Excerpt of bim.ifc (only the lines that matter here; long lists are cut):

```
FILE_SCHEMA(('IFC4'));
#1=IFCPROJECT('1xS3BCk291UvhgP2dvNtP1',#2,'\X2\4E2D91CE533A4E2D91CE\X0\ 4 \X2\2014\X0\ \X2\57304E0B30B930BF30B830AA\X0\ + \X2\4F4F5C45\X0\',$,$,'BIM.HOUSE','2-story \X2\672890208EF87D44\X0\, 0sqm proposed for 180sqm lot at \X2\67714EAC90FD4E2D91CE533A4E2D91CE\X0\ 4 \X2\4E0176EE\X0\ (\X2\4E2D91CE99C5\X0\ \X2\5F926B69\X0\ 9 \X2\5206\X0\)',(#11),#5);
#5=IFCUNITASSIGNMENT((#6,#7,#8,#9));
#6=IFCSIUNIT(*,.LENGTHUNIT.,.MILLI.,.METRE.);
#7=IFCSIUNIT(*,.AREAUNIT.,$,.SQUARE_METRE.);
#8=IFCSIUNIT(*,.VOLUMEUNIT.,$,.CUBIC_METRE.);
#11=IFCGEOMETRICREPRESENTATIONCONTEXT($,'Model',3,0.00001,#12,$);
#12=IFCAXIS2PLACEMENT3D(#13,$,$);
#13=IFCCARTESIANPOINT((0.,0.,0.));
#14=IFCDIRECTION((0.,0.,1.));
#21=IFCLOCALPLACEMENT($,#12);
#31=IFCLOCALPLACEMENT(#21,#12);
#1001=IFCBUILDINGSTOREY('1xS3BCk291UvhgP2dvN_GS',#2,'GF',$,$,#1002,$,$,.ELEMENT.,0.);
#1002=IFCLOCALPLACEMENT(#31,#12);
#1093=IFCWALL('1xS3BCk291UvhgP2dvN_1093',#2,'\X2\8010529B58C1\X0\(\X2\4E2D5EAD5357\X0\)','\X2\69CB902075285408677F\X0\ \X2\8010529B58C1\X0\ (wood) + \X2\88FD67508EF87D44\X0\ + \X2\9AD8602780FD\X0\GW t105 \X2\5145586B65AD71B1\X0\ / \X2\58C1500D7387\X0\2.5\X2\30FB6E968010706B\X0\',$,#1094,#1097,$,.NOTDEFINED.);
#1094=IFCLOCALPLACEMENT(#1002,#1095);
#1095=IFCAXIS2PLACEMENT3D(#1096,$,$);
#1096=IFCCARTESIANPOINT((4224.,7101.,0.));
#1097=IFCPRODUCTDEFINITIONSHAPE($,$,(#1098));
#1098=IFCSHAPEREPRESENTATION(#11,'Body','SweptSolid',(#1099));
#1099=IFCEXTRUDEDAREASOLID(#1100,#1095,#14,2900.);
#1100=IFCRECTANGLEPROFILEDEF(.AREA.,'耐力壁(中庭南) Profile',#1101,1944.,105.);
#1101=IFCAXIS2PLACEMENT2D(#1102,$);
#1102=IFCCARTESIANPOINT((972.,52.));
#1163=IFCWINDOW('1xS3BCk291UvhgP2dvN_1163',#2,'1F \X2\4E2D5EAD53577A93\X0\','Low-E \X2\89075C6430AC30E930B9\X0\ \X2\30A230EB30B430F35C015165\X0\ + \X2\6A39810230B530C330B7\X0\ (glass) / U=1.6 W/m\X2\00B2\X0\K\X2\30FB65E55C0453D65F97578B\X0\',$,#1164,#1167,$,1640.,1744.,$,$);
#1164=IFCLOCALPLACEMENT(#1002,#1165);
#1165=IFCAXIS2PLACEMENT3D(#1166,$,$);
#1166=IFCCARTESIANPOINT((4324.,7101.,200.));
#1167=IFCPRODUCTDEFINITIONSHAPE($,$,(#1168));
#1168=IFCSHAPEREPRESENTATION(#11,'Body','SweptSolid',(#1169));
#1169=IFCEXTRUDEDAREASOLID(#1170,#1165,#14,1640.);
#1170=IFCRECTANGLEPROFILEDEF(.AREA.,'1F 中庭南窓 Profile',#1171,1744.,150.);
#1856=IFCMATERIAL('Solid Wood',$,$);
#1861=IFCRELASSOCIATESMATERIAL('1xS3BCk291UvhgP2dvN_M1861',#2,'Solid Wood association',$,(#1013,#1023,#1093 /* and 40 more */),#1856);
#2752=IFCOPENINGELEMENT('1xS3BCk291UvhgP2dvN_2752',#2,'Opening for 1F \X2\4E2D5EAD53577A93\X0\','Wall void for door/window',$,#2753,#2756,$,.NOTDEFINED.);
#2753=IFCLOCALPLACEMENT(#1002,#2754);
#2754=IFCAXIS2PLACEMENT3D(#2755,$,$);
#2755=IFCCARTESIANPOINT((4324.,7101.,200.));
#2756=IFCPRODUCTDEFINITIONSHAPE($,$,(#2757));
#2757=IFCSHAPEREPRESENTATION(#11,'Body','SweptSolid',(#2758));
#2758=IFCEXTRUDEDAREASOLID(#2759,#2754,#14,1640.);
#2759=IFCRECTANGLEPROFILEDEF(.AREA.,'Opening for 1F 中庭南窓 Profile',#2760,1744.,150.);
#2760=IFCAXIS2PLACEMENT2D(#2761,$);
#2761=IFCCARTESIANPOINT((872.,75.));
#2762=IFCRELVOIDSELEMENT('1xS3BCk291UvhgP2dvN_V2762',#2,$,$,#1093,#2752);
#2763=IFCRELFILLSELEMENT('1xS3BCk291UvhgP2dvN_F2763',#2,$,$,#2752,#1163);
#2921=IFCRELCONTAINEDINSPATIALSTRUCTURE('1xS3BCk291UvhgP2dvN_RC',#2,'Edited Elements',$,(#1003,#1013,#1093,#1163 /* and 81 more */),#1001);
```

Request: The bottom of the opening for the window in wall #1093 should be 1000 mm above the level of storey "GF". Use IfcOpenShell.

```python
import numpy as np
import ifcopenshell
import ifcopenshell.api.geometry
import ifcopenshell.geom
import ifcopenshell.util.element
import ifcopenshell.util.placement
import ifcopenshell.util.shape
import ifcopenshell.util.unit

model = ifcopenshell.open("bim.ifc")
unit_scale = ifcopenshell.util.unit.calculate_unit_scale(model)

window = model.by_guid("1xS3BCk291UvhgP2dvN_1163")
opening = window.FillsVoids[0].RelatingOpeningElement
storey = ifcopenshell.util.element.get_container(window, ifc_class="IfcBuildingStorey")
level = ifcopenshell.util.placement.get_local_placement(storey.ObjectPlacement)[2, 3]

# The opening's origin need not be at the sill, so measure its lowest point.
shape = ifcopenshell.geom.create_shape(ifcopenshell.geom.settings(), opening)
bottom = ifcopenshell.util.shape.get_shape_bottom_elevation(shape, shape.geometry) / unit_scale
dz = level + 1 / unit_scale - bottom

shift = np.array([0.0, 0.0, dz])
# The window is not placed relative to its opening, so move both.
for product in (opening, window):
    matrix = ifcopenshell.util.placement.get_local_placement(product.ObjectPlacement)
    matrix[:3, 3] += shift
    ifcopenshell.api.geometry.edit_object_placement(model, product=product, matrix=matrix, is_si=False)

print(f"moved by {dz * unit_scale:+.3f} m")

model.write("bim_updated.ifc")
```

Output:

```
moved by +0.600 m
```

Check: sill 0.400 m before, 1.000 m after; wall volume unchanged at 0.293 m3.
